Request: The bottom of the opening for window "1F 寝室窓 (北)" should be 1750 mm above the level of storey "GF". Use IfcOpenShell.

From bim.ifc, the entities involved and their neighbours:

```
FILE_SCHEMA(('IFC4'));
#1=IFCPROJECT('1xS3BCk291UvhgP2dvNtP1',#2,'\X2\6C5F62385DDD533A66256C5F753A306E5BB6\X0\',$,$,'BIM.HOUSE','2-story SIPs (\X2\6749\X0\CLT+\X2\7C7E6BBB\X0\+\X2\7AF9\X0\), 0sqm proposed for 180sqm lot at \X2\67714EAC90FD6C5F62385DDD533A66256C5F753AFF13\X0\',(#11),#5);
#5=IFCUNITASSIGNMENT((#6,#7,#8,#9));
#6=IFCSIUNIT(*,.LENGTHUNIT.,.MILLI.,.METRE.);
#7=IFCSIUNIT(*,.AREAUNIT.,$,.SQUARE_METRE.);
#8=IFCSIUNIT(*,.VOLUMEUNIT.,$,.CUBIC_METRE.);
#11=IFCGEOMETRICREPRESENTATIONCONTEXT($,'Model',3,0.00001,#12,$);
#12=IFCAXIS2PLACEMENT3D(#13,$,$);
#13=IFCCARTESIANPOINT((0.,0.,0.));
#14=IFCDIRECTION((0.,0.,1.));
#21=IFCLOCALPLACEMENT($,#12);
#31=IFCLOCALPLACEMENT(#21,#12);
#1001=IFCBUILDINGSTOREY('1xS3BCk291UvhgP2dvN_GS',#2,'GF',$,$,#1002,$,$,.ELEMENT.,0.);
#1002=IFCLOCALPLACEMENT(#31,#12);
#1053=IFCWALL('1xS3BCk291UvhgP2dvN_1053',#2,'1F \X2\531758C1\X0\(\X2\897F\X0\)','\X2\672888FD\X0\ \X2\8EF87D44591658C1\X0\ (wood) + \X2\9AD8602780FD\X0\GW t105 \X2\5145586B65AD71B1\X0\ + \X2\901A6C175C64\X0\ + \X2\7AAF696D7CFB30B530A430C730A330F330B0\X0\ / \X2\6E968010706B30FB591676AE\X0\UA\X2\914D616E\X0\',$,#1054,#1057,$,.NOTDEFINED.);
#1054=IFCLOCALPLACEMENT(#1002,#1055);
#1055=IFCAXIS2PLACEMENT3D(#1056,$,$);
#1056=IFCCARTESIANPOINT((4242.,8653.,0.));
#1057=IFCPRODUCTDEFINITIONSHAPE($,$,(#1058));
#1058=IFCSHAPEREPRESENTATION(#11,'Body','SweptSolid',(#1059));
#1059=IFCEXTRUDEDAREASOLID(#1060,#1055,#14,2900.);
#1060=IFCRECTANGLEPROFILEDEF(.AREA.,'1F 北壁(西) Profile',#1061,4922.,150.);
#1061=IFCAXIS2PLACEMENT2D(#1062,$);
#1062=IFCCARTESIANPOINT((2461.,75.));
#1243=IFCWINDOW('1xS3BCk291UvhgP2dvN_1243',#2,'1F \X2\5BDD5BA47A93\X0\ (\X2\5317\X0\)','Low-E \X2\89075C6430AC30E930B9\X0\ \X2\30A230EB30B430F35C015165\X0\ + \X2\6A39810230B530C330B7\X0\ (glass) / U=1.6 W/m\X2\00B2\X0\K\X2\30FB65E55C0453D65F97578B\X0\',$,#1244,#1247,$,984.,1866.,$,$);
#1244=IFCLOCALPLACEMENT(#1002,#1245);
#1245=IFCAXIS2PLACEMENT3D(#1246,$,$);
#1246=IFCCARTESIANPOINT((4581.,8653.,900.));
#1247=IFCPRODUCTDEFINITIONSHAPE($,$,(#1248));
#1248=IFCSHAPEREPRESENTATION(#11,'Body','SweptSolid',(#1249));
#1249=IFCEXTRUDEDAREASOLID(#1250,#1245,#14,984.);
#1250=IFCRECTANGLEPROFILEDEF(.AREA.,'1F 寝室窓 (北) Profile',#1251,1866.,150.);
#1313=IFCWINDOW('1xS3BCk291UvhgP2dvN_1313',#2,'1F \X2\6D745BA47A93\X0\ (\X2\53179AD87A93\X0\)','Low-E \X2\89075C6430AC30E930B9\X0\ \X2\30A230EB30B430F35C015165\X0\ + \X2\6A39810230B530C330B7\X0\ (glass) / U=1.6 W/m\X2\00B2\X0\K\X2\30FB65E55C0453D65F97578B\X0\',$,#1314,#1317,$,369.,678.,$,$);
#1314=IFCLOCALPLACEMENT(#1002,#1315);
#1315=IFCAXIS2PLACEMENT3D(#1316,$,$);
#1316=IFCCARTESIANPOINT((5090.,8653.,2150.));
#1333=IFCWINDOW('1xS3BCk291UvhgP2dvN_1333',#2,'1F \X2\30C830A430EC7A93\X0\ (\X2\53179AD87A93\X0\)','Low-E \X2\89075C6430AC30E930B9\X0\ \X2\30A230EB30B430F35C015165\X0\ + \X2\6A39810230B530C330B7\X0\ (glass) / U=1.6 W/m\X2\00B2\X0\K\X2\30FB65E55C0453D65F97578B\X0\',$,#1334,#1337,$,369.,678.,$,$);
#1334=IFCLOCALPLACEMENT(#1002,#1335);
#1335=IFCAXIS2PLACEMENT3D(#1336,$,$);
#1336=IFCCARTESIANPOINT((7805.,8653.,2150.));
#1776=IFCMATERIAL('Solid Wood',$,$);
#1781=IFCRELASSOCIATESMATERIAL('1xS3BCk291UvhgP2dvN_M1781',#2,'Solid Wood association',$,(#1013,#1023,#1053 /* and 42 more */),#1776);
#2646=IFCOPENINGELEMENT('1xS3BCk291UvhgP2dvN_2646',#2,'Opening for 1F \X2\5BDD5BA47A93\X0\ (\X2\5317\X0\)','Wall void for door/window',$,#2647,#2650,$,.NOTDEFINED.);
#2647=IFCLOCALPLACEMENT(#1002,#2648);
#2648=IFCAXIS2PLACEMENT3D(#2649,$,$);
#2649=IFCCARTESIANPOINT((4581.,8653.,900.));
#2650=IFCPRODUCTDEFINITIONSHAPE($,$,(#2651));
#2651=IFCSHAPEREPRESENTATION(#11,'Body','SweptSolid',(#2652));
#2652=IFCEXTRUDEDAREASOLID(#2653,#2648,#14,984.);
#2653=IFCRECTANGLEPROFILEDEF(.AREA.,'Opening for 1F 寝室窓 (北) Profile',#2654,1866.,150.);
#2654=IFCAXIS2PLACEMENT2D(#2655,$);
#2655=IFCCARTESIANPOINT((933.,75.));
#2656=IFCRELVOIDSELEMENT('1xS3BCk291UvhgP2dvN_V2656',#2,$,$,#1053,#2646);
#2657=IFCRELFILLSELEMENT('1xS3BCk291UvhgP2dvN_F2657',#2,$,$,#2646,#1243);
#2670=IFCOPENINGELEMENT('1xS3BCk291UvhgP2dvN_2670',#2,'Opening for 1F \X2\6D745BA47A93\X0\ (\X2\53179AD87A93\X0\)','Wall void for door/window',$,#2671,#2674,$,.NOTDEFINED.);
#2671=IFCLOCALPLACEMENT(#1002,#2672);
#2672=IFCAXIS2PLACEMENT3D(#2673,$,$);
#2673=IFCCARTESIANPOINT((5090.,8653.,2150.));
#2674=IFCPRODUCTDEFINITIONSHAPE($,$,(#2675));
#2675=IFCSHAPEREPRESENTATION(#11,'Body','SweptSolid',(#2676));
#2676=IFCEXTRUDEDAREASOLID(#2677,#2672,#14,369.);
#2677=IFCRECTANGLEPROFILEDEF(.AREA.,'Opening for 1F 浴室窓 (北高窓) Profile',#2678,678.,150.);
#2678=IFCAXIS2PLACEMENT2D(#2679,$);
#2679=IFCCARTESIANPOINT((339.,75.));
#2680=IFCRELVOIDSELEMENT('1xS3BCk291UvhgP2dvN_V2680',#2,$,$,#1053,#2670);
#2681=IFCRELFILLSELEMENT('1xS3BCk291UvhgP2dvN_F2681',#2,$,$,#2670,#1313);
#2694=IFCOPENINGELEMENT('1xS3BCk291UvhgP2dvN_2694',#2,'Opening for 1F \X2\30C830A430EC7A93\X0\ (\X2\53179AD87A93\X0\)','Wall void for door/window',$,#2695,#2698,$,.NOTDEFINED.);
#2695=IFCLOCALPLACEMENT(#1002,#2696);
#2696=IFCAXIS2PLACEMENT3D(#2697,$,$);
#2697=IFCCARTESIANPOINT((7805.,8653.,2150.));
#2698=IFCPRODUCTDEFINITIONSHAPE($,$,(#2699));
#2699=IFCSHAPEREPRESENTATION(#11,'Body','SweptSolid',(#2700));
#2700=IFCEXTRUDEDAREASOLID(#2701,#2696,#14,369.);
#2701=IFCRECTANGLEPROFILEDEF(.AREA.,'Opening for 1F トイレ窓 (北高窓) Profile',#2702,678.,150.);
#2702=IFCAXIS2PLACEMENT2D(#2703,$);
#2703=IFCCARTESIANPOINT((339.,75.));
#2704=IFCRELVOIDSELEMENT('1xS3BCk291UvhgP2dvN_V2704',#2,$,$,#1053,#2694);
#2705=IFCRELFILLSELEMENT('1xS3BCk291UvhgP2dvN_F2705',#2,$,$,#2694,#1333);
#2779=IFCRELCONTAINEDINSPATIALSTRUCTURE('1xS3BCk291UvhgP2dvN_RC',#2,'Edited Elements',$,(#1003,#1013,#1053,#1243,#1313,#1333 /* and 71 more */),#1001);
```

```python
import numpy as np
import ifcopenshell
import ifcopenshell.api.geometry
import ifcopenshell.geom
import ifcopenshell.util.element
import ifcopenshell.util.placement
import ifcopenshell.util.shape
import ifcopenshell.util.unit

model = ifcopenshell.open("bim.ifc")
unit_scale = ifcopenshell.util.unit.calculate_unit_scale(model)

window = model.by_id(1243)
opening = window.FillsVoids[0].RelatingOpeningElement
storey = ifcopenshell.util.element.get_container(window, ifc_class="IfcBuildingStorey")
level = ifcopenshell.util.placement.get_local_placement(storey.ObjectPlacement)[2, 3]

# The opening's origin need not be at the sill, so measure its lowest point.
shape = ifcopenshell.geom.create_shape(ifcopenshell.geom.settings(), opening)
bottom = ifcopenshell.util.shape.get_shape_bottom_elevation(shape, shape.geometry) / unit_scale
dz = level + 1750.0 - bottom

shift = np.array([0.0, 0.0, dz])
# The window is not placed relative to its opening, so move both.
for product in (opening, window):
    matrix = ifcopenshell.util.placement.get_local_placement(product.ObjectPlacement)
    matrix[:3, 3] += shift
    ifcopenshell.api.geometry.edit_object_placement(model, product=product, matrix=matrix, is_si=False)

print(f"moved by {dz * unit_scale:+.3f} m")

model.write("bim-out.ifc")
```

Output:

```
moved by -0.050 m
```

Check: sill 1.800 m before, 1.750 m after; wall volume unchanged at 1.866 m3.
